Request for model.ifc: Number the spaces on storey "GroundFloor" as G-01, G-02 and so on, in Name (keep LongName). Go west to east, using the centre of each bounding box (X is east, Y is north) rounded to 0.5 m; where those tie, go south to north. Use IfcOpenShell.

First a look at what the model holds.

```python
import ifcopenshell
import ifcopenshell.util.element
import ifcopenshell.util.placement

model = ifcopenshell.open("model.ifc")
print(model.schema)
storey = next(s for s in model.by_type("IfcBuildingStorey") if s.Name == "GroundFloor")
spaces = [e for e in ifcopenshell.util.element.get_decomposition(storey) if e.is_a("IfcSpace")]
for e in sorted(spaces, key=lambda e: e.id()):
    origin = ifcopenshell.util.placement.get_local_placement(e.ObjectPlacement)[:3, 3]
    print(e.id(), e.Name, e.LongName, origin.round(2) + 0.0, sep=" | ")
```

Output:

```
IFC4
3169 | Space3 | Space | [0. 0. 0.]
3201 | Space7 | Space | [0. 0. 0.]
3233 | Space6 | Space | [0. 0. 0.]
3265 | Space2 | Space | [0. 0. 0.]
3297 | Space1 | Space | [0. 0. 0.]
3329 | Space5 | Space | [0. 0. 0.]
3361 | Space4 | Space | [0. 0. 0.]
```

```python
import ifcopenshell
import ifcopenshell.geom
import ifcopenshell.util.element
import ifcopenshell.util.shape

model = ifcopenshell.open("model.ifc")
settings = ifcopenshell.geom.settings()
settings.set("use-world-coords", True)


def centre(element):
    shape = ifcopenshell.geom.create_shape(settings, element)
    return ifcopenshell.util.shape.get_bbox_centroid(shape.geometry)


storey = next(s for s in model.by_type("IfcBuildingStorey") if s.Name == "GroundFloor")
spaces = [e for e in ifcopenshell.util.element.get_decomposition(storey) if e.is_a("IfcSpace")]

# Insertion points can sit at a corner or the storey origin, so sort by the geometry (in metres).
centres = {e: centre(e) for e in spaces}
spaces.sort(key=lambda e: (round(centres[e][0] / 0.5), centres[e][1]))

for i, e in enumerate(spaces, start=1):
    number = f"G-{i:02d}"
    e.Name = number
    print(e.id(), number)

model.write("model_updated.ifc")
```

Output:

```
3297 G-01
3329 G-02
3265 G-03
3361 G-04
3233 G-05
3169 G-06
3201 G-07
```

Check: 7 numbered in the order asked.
